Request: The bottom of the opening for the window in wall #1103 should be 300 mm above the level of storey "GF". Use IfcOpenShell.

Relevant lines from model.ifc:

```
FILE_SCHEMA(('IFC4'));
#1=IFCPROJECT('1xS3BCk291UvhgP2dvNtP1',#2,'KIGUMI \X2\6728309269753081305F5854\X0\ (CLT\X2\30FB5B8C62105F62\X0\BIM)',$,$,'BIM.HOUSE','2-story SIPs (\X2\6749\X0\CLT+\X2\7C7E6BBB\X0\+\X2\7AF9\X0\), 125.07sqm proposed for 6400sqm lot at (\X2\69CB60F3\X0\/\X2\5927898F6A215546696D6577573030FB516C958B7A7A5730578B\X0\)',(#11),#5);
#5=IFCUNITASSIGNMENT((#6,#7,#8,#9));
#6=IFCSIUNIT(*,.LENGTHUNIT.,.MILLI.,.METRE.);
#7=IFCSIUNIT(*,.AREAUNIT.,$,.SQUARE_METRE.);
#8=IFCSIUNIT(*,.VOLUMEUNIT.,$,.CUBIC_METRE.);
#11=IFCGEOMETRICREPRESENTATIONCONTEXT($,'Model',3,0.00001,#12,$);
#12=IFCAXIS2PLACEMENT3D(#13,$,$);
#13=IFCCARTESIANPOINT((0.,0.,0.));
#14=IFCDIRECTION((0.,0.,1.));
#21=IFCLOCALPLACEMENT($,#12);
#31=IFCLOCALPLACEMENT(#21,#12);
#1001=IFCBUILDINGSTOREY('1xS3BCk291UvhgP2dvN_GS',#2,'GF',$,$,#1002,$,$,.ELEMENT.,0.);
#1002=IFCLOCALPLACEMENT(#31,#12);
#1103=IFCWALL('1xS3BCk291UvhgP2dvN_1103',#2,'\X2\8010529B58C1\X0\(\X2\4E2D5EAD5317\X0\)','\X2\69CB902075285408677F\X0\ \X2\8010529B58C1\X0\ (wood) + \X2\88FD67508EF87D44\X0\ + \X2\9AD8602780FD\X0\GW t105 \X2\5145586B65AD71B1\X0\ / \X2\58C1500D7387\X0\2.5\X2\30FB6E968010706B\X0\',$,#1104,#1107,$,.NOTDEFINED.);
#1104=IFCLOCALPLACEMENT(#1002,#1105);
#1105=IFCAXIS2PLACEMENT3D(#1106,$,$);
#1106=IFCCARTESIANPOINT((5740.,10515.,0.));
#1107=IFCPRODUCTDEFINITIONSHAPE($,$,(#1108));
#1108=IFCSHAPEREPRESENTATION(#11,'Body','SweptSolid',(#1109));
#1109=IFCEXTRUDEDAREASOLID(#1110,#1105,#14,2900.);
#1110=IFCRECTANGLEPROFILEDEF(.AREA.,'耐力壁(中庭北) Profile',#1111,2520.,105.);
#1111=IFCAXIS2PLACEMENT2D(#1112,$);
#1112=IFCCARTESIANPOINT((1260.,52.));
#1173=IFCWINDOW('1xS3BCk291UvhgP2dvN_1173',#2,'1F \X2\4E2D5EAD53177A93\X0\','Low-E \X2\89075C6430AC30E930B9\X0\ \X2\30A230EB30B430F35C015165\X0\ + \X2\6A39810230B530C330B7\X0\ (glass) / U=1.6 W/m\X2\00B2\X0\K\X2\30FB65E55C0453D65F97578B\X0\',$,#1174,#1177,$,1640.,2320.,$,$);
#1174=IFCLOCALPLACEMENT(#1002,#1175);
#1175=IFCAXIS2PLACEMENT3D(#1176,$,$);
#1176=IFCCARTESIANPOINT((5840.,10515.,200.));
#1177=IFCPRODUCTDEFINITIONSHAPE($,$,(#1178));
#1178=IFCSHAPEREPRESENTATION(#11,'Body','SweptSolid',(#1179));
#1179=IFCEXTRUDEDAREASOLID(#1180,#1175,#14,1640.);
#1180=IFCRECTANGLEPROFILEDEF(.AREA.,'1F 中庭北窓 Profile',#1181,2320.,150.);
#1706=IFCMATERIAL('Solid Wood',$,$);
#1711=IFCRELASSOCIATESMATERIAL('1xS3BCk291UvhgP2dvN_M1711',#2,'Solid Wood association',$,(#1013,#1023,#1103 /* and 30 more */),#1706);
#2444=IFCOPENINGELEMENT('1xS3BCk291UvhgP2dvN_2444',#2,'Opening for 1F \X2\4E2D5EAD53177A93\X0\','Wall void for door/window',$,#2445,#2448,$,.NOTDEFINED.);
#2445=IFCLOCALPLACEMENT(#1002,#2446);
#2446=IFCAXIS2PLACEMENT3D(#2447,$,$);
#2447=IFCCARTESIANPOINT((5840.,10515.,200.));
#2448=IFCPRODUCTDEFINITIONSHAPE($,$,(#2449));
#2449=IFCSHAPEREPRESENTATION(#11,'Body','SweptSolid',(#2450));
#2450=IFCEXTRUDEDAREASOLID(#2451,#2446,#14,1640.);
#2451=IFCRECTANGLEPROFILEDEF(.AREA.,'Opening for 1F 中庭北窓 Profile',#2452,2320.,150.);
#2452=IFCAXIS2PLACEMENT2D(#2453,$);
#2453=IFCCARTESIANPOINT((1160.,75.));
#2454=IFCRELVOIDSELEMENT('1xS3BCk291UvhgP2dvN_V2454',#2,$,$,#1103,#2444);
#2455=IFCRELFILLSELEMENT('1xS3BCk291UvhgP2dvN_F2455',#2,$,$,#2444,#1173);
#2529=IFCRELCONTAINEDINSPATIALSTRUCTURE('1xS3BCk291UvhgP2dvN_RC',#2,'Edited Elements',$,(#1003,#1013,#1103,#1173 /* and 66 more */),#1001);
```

```python
import numpy as np
import ifcopenshell
import ifcopenshell.api.geometry
import ifcopenshell.geom
import ifcopenshell.util.element
import ifcopenshell.util.placement
import ifcopenshell.util.shape
import ifcopenshell.util.unit

model = ifcopenshell.open("model.ifc")
unit_scale = ifcopenshell.util.unit.calculate_unit_scale(model)

window = model.by_guid("1xS3BCk291UvhgP2dvN_1173")
opening = window.FillsVoids[0].RelatingOpeningElement
storey = ifcopenshell.util.element.get_container(window, ifc_class="IfcBuildingStorey")
level = ifcopenshell.util.placement.get_local_placement(storey.ObjectPlacement)[2, 3]

# The opening's origin need not be at the sill, so measure its lowest point.
shape = ifcopenshell.geom.create_shape(ifcopenshell.geom.settings(), opening)
bottom = ifcopenshell.util.shape.get_shape_bottom_elevation(shape, shape.geometry) / unit_scale
dz = level + 0.3 / unit_scale - bottom

shift = np.array([0.0, 0.0, dz])
# The window is not placed relative to its opening, so move both.
for product in (opening, window):
    matrix = ifcopenshell.util.placement.get_local_placement(product.ObjectPlacement)
    matrix[:3, 3] += shift
    ifcopenshell.api.geometry.edit_object_placement(model, product=product, matrix=matrix, is_si=False)

print(f"moved by {dz * unit_scale:+.3f} m")

model.write("model_edited.ifc")
```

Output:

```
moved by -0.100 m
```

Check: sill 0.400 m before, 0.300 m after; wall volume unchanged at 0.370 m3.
